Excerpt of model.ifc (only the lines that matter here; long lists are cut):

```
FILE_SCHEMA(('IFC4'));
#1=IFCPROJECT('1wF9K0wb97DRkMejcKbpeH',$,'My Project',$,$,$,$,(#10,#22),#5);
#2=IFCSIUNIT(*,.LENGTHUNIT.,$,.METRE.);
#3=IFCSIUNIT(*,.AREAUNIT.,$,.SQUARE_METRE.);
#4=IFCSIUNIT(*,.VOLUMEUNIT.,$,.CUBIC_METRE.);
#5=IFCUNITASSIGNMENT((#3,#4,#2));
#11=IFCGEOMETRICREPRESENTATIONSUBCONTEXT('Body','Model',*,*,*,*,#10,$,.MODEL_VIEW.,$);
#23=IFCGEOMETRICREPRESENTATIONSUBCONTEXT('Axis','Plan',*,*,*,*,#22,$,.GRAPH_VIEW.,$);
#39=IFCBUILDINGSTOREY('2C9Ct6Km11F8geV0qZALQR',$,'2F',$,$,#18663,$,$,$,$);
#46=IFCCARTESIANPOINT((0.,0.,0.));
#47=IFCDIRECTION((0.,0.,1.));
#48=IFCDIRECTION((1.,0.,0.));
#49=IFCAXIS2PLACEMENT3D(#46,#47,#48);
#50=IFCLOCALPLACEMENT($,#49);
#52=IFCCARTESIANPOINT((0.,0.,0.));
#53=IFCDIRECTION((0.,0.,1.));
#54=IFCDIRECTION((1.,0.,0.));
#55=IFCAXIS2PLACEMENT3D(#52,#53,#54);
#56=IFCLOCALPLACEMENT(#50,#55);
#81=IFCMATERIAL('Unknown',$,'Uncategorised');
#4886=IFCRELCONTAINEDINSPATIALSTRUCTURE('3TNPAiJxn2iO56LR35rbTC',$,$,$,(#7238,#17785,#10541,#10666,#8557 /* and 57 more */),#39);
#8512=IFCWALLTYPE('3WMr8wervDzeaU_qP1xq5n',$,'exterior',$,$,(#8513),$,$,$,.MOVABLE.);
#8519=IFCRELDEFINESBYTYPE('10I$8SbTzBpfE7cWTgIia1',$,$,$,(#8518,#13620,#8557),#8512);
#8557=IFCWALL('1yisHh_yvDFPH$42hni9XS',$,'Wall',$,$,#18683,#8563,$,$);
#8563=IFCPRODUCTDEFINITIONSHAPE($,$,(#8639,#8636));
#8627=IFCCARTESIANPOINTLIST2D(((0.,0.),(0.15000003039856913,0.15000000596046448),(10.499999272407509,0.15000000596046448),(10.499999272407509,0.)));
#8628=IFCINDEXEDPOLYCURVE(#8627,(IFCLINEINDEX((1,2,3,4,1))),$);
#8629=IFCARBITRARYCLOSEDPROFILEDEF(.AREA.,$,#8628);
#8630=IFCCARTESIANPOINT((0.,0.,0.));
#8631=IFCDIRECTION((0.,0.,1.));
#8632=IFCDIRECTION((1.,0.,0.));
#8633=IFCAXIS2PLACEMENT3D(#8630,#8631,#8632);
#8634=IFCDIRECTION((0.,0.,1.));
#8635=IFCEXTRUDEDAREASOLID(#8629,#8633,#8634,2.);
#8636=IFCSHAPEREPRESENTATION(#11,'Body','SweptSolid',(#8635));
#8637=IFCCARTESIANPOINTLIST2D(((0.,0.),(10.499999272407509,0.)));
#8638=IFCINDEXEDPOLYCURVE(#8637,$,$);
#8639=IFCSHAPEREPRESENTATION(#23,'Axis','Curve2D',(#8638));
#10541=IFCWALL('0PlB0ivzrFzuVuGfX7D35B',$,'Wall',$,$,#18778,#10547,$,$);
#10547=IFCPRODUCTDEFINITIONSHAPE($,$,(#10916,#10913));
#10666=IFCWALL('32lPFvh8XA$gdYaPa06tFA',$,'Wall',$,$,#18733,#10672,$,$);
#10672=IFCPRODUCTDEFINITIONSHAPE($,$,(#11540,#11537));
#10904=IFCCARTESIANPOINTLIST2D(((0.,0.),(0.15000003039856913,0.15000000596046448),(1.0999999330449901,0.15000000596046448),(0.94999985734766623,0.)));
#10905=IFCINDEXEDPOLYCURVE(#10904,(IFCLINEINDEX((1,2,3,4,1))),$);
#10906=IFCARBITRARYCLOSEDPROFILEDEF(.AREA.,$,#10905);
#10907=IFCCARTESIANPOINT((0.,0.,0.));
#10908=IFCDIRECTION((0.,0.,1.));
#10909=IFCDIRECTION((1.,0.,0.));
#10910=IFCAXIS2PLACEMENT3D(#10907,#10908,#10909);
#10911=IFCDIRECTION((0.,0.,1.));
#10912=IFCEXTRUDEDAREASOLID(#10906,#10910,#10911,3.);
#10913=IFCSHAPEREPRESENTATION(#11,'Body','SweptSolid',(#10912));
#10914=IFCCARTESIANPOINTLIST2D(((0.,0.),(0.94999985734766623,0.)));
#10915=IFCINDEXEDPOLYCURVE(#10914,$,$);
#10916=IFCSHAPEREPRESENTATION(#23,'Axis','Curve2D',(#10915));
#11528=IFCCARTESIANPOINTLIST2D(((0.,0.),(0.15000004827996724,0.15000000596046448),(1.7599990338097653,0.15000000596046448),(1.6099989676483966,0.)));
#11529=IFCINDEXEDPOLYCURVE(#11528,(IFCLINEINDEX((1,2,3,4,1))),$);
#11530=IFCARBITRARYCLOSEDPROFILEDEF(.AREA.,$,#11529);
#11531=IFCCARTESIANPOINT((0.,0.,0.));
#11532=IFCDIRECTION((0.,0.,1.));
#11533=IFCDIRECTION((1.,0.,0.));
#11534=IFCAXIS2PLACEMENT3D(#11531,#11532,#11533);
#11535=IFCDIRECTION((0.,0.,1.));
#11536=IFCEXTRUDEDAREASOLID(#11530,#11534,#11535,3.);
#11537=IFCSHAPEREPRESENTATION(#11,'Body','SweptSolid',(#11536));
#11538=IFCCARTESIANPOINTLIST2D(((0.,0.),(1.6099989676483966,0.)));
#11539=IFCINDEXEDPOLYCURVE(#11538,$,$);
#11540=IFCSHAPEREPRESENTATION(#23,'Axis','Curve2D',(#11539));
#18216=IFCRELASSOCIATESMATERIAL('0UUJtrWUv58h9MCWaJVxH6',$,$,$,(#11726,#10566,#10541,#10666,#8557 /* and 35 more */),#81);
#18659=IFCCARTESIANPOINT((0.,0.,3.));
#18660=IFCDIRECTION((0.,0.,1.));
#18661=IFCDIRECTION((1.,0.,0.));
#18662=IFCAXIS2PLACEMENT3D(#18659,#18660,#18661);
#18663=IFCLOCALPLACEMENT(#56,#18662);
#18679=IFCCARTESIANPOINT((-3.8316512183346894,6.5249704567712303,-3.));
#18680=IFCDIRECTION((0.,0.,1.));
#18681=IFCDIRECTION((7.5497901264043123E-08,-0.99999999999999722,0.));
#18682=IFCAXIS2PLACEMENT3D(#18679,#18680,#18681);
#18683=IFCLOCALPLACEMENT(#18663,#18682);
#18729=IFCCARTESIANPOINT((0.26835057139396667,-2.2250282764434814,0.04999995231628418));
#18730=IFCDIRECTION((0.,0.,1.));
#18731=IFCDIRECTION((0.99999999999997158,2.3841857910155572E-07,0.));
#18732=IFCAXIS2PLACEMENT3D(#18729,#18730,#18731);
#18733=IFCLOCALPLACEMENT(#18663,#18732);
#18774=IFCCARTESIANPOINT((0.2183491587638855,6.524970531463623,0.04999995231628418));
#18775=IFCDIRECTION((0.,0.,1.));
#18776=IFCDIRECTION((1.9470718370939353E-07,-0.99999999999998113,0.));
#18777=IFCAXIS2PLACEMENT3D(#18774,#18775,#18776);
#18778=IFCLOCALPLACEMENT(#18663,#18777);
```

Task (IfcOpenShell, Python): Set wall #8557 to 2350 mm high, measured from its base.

```python
import ifcopenshell
import ifcopenshell.geom
import ifcopenshell.util.representation
import ifcopenshell.util.shape
import ifcopenshell.util.unit

model = ifcopenshell.open("model.ifc")
unit_scale = ifcopenshell.util.unit.calculate_unit_scale(model)
settings = ifcopenshell.geom.settings()


def volume(element):
    """Net volume in cubic metres, openings subtracted."""
    shape = ifcopenshell.geom.create_shape(settings, element)
    return ifcopenshell.util.shape.get_volume(shape.geometry)


wall = model.by_id(8557)
before = volume(wall)

body = ifcopenshell.util.representation.get_representation(wall, "Model", "Body")
solid = body.Items[0]
old_height = solid.Depth
solid.Depth = 2.35 / unit_scale
after = volume(wall)

print(f"height {old_height:g} -> {solid.Depth:g}, volume {before:.3f} -> {after:.3f} m3")

model.write("model_edited.ifc")
```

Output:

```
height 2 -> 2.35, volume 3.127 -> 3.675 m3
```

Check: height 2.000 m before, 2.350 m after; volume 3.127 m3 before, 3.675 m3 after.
